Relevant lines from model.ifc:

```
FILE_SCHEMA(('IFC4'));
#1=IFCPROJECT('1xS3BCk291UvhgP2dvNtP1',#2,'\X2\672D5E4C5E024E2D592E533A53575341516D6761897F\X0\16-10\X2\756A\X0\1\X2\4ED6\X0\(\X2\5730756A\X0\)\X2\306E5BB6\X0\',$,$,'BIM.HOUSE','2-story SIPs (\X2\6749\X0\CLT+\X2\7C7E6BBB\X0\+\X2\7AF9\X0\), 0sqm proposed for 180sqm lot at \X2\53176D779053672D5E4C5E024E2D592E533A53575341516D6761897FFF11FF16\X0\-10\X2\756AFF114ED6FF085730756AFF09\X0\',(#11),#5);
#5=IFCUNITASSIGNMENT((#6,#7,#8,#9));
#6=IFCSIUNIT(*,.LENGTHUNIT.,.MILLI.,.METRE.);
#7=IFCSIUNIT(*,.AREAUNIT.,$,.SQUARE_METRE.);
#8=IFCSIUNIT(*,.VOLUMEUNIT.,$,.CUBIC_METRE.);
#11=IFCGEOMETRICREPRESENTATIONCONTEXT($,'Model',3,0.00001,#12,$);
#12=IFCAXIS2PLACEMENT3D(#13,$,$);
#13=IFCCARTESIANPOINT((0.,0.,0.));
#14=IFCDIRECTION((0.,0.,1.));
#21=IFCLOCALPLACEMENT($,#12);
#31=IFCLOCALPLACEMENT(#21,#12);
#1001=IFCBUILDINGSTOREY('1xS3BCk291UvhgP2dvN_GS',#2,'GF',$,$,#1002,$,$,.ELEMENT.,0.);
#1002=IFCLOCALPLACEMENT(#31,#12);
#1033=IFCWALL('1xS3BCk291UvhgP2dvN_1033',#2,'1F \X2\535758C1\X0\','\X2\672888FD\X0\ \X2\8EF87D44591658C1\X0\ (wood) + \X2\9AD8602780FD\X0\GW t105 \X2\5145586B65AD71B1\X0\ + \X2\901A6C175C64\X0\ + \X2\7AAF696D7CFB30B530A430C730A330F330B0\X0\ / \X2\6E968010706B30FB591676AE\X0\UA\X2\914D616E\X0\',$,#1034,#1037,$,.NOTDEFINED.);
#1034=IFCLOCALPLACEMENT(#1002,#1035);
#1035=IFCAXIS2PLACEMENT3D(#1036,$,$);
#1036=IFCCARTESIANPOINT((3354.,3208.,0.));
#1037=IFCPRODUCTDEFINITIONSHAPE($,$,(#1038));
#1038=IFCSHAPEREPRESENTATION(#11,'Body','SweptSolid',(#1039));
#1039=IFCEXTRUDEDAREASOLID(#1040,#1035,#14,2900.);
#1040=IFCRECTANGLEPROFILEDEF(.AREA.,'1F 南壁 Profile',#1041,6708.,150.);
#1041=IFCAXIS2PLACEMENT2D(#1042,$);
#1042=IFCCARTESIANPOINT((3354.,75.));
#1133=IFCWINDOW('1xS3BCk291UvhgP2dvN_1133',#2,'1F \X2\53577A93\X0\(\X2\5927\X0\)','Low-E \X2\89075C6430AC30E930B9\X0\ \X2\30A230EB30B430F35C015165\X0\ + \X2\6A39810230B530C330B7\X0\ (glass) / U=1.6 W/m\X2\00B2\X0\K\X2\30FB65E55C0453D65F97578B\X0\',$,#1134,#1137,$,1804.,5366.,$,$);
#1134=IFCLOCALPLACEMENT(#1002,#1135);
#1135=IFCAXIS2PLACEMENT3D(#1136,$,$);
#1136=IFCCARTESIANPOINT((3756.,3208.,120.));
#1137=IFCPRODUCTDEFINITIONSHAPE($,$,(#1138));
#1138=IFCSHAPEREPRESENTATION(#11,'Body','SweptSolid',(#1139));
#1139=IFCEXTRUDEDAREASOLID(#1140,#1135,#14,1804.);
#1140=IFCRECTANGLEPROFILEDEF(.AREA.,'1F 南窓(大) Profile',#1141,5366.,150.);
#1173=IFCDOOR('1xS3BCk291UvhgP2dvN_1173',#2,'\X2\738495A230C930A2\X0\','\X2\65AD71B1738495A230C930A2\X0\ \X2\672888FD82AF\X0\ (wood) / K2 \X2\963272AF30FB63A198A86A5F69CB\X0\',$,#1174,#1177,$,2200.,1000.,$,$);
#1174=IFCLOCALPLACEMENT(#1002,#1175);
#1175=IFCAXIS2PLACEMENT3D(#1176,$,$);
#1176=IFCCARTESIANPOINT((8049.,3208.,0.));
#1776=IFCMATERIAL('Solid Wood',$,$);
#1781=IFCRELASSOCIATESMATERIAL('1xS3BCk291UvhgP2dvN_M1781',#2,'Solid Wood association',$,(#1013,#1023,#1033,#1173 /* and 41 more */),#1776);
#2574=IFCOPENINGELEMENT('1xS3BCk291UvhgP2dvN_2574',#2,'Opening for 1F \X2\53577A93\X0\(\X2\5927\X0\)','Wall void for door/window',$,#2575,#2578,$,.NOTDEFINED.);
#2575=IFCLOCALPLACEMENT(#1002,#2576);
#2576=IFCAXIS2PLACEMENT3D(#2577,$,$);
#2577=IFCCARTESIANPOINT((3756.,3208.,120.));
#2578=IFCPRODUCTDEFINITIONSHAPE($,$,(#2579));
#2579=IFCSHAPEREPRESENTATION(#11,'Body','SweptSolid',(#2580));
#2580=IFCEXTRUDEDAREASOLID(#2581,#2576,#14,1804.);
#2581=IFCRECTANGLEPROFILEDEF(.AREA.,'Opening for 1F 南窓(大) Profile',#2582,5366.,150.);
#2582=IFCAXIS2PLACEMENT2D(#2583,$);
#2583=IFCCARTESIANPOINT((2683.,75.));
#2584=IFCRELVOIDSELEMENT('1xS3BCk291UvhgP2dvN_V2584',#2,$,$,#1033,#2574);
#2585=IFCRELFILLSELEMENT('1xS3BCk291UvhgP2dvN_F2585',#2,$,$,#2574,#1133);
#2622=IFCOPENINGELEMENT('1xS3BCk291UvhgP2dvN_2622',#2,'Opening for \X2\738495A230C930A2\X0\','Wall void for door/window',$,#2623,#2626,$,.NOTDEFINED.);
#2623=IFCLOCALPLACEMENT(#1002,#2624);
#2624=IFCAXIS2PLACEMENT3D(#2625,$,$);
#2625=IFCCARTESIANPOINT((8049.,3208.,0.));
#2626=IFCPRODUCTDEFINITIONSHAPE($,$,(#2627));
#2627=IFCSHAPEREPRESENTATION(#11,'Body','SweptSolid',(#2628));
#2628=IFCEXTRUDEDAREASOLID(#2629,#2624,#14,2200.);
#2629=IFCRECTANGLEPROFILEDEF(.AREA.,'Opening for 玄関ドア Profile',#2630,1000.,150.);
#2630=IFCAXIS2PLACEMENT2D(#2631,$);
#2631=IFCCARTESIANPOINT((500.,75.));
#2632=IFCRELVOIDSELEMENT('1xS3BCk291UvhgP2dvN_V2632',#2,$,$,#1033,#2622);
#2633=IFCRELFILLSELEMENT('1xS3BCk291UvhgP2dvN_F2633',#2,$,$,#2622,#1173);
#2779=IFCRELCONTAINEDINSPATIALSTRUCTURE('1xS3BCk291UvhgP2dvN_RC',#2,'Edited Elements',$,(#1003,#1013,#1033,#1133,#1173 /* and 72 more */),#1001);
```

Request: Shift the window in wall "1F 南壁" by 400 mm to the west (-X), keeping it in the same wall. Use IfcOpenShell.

```python
import ifcopenshell
import ifcopenshell.api.geometry
import ifcopenshell.util.placement

model = ifcopenshell.open("model.ifc")

window = model.by_guid("1xS3BCk291UvhgP2dvN_1133")
opening = window.FillsVoids[0].RelatingOpeningElement
wall = opening.VoidsElements[0].RelatingBuildingElement

wall_matrix = ifcopenshell.util.placement.get_local_placement(wall.ObjectPlacement)
shift = wall_matrix[:3, 0] * -400.0
before = ifcopenshell.util.placement.get_local_placement(window.ObjectPlacement)[:3, 3].copy()

# The window is not placed relative to its opening, so move both.
for product in (opening, window):
    matrix = ifcopenshell.util.placement.get_local_placement(product.ObjectPlacement)
    matrix[:3, 3] += shift
    ifcopenshell.api.geometry.edit_object_placement(model, product=product, matrix=matrix, is_si=False)

after = ifcopenshell.util.placement.get_local_placement(window.ObjectPlacement)[:3, 3]
print("window moved by", (after - before).round(3) + 0.0)

model.write("model_updated.ifc")
```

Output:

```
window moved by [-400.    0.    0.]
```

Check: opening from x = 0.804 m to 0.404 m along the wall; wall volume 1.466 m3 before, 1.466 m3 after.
